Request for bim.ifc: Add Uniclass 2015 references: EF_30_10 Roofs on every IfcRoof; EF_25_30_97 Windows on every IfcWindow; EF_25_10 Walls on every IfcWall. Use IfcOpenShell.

First a look at what the model holds.

```python
import ifcopenshell

model = ifcopenshell.open("bim.ifc")
print(model.schema)
print("classifications:", [c.Name for c in model.by_type("IfcClassification")])
for ifc_class in ("IfcDoor", "IfcRoof", "IfcStair", "IfcWall", "IfcWindow"):
    print(ifc_class, len(model.by_type(ifc_class)))
```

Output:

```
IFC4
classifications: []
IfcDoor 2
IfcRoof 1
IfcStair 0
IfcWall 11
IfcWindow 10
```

```python
import ifcopenshell
import ifcopenshell.api.classification

model = ifcopenshell.open("bim.ifc")

system = ifcopenshell.api.classification.add_classification(model, classification="Uniclass 2015")

codes = {
    "IfcRoof": ("EF_30_10", "Roofs"),
    "IfcWindow": ("EF_25_30_97", "Windows"),
    "IfcWall": ("EF_25_10", "Walls"),
}
for ifc_class, (code, name) in codes.items():
    products = model.by_type(ifc_class)
    ifcopenshell.api.classification.add_reference(
        model, products=products, classification=system, identification=code, name=name
    )
    print(code, len(products))

model.write("bim_edited.ifc")
```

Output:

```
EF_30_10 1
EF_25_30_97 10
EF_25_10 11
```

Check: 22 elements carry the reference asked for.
